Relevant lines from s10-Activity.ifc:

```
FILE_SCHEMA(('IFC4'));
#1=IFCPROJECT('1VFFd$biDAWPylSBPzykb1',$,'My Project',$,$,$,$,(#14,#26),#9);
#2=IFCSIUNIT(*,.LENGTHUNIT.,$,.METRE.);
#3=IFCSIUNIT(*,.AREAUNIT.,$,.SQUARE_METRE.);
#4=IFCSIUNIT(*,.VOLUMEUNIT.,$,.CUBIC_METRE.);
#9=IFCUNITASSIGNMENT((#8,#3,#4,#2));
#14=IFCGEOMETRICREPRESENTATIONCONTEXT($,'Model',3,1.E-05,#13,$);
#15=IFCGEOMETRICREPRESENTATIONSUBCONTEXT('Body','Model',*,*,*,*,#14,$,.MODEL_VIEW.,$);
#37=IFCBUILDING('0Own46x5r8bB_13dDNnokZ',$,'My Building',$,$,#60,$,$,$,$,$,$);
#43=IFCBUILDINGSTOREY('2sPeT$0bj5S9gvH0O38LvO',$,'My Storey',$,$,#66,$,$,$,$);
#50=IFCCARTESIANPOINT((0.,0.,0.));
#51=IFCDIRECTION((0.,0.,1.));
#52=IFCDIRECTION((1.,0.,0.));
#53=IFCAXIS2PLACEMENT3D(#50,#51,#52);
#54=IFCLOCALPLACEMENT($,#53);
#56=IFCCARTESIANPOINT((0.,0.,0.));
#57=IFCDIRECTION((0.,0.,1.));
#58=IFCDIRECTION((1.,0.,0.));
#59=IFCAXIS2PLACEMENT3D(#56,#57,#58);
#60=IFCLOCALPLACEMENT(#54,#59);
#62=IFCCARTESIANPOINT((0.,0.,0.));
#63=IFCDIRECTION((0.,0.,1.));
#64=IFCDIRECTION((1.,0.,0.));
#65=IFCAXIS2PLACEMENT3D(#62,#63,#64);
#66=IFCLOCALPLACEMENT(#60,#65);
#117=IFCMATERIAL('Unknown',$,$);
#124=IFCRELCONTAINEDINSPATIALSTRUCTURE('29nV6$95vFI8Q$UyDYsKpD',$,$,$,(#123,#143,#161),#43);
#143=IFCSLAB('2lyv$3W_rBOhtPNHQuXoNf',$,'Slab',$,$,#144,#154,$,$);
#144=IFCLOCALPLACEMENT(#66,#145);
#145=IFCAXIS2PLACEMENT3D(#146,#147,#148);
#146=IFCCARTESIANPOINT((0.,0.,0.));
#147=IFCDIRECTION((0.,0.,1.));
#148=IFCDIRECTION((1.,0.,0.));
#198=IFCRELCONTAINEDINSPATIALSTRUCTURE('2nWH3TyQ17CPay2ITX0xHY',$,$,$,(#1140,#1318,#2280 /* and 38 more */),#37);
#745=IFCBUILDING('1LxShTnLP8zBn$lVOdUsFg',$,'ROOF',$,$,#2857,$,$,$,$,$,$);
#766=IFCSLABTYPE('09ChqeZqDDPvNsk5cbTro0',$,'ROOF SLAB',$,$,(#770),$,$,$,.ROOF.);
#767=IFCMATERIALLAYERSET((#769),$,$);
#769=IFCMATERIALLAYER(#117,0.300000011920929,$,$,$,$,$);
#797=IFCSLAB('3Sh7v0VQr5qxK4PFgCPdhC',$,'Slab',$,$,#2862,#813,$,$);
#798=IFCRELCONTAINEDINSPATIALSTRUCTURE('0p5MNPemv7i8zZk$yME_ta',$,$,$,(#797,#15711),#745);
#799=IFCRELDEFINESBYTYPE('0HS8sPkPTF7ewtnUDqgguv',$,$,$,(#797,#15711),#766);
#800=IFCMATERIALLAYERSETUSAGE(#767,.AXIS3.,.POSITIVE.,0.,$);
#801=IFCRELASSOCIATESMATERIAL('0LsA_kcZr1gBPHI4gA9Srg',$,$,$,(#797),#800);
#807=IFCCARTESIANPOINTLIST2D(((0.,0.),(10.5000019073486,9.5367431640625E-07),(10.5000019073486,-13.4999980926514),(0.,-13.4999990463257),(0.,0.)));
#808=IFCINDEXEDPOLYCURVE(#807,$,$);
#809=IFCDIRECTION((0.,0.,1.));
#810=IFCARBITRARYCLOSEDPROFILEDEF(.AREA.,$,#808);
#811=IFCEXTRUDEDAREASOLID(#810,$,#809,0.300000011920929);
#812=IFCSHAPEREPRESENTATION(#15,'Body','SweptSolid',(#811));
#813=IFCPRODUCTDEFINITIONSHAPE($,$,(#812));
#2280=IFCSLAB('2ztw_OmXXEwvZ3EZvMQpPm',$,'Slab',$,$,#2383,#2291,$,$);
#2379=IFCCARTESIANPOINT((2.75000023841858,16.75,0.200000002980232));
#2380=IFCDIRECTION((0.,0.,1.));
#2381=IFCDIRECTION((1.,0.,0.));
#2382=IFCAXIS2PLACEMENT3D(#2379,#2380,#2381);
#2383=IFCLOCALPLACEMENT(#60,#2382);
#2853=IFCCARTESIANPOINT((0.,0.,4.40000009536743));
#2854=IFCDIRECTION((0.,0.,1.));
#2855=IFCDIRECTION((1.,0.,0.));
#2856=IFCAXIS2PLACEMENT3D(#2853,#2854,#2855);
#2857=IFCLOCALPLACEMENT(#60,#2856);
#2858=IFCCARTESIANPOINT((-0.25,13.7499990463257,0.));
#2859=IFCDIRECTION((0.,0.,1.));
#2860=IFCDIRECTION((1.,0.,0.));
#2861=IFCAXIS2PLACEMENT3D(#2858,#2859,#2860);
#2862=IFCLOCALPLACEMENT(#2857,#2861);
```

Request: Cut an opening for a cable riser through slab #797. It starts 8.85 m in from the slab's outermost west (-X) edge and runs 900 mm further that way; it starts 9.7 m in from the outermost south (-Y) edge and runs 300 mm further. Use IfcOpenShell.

```python
import numpy as np
import ifcopenshell
import ifcopenshell.api.feature
import ifcopenshell.api.geometry
import ifcopenshell.api.root
import ifcopenshell.geom
import ifcopenshell.util.placement
import ifcopenshell.util.representation
import ifcopenshell.util.shape
import ifcopenshell.util.unit

model = ifcopenshell.open("s10-Activity.ifc")
unit_scale = ifcopenshell.util.unit.calculate_unit_scale(model)
settings = ifcopenshell.geom.settings()


def volume(element):
    """Net volume in cubic metres, openings subtracted."""
    shape = ifcopenshell.geom.create_shape(settings, element)
    return ifcopenshell.util.shape.get_volume(shape.geometry)


slab = model.by_guid("3Sh7v0VQr5qxK4PFgCPdhC")
before = volume(slab)

# Extent in the slab's own axes, in metres. The edges named are its -X and -Y sides.
slab_shape = ifcopenshell.geom.create_shape(settings, slab)
vertices = ifcopenshell.util.shape.get_vertices(slab_shape.geometry)
x_min, y_min, bottom = vertices.min(axis=0)
top = vertices[:, 2].max()

opening = ifcopenshell.api.root.create_entity(model, ifc_class="IfcOpeningElement", name="Cable riser opening", predefined_type="OPENING")
context = ifcopenshell.util.representation.get_context(model, "Model", "Body", "MODEL_VIEW")
width, depth = 0.9, 0.3
outline = [(0.0, 0.0), (width, 0.0), (width, depth), (0.0, depth), (0.0, 0.0)]
# Overshoot both faces by 50 mm so the cut is clean.
shape = ifcopenshell.api.geometry.add_slab_representation(
    model, context=context, depth=top - bottom + 0.1, polyline=outline
)
ifcopenshell.api.geometry.assign_representation(model, product=opening, representation=shape)

matrix = ifcopenshell.util.placement.get_local_placement(slab.ObjectPlacement)
matrix[:, 3] = matrix @ np.append(np.array([x_min + 8.85, y_min + 9.7, bottom - 0.05]) / unit_scale, 1.0)
ifcopenshell.api.geometry.edit_object_placement(model, product=opening, matrix=matrix, is_si=False)
ifcopenshell.api.feature.add_feature(model, feature=opening, element=slab)

after = volume(slab)

print(f"slab volume {before:.3f} -> {after:.3f} m3")

model.write("s10-Activity_v2.ifc")
```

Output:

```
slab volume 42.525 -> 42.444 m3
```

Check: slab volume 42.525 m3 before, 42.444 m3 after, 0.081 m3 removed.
